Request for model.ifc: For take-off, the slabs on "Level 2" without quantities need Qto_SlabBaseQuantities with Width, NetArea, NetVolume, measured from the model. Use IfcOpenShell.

First a look at what the model holds.

```python
import ifcopenshell
import ifcopenshell.util.element
import ifcopenshell.util.unit

model = ifcopenshell.open("model.ifc")
print(model.schema)
for unit_type in ("LENGTHUNIT", "AREAUNIT", "VOLUMEUNIT"):
    print(unit_type, ifcopenshell.util.unit.calculate_unit_scale(model, unit_type))
storey = next(s for s in model.by_type("IfcBuildingStorey") if s.Name == "Level 2")
slabs = [e for e in ifcopenshell.util.element.get_decomposition(storey) if e.is_a("IfcSlab")]
for e in sorted(slabs, key=lambda e: e.id()):
    print(e.id(), e.is_a(), e.Name, list(ifcopenshell.util.element.get_psets(e, qtos_only=True)), sep=" | ")
```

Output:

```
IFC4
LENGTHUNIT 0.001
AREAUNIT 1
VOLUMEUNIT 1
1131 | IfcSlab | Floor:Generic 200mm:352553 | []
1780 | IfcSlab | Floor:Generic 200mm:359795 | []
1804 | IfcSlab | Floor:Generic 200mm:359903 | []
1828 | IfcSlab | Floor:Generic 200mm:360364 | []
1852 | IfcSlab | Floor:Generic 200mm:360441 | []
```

```python
import ifcopenshell
import ifcopenshell.api.pset
import ifcopenshell.geom
import ifcopenshell.util.element
import ifcopenshell.util.shape
import ifcopenshell.util.unit

model = ifcopenshell.open("model.ifc")
unit_scale = ifcopenshell.util.unit.calculate_unit_scale(model)
area_scale = ifcopenshell.util.unit.calculate_unit_scale(model, "AREAUNIT")
volume_scale = ifcopenshell.util.unit.calculate_unit_scale(model, "VOLUMEUNIT")
settings = ifcopenshell.geom.settings()

storey = next(s for s in model.by_type("IfcBuildingStorey") if s.Name == "Level 2")
slabs = [e for e in ifcopenshell.util.element.get_decomposition(storey) if e.is_a("IfcSlab")]

for e in sorted(slabs, key=lambda e: e.id()):
    if ifcopenshell.util.element.get_psets(e, qtos_only=True, should_inherit=False):
        continue
    # Geometry comes back in metres, in the element's own axes.
    shape = ifcopenshell.geom.create_shape(settings, e)
    values = {
        "Width": ifcopenshell.util.shape.get_z(shape.geometry) / unit_scale,
        "NetArea": ifcopenshell.util.shape.get_footprint_area(shape.geometry) / area_scale,
        "NetVolume": ifcopenshell.util.shape.get_volume(shape.geometry) / volume_scale,
    }
    qto = ifcopenshell.api.pset.add_qto(model, product=e, name="Qto_SlabBaseQuantities")
    ifcopenshell.api.pset.edit_qto(model, qto=qto, properties=values)
    print(e.id(), {k: round(v, 3) for k, v in values.items()})

model.write("model_v2.ifc")
```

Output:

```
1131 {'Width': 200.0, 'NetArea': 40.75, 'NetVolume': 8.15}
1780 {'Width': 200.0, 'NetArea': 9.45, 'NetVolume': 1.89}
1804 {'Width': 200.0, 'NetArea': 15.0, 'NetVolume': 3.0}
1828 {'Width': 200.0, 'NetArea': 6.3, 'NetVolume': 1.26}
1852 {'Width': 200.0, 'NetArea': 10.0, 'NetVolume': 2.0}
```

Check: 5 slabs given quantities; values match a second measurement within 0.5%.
